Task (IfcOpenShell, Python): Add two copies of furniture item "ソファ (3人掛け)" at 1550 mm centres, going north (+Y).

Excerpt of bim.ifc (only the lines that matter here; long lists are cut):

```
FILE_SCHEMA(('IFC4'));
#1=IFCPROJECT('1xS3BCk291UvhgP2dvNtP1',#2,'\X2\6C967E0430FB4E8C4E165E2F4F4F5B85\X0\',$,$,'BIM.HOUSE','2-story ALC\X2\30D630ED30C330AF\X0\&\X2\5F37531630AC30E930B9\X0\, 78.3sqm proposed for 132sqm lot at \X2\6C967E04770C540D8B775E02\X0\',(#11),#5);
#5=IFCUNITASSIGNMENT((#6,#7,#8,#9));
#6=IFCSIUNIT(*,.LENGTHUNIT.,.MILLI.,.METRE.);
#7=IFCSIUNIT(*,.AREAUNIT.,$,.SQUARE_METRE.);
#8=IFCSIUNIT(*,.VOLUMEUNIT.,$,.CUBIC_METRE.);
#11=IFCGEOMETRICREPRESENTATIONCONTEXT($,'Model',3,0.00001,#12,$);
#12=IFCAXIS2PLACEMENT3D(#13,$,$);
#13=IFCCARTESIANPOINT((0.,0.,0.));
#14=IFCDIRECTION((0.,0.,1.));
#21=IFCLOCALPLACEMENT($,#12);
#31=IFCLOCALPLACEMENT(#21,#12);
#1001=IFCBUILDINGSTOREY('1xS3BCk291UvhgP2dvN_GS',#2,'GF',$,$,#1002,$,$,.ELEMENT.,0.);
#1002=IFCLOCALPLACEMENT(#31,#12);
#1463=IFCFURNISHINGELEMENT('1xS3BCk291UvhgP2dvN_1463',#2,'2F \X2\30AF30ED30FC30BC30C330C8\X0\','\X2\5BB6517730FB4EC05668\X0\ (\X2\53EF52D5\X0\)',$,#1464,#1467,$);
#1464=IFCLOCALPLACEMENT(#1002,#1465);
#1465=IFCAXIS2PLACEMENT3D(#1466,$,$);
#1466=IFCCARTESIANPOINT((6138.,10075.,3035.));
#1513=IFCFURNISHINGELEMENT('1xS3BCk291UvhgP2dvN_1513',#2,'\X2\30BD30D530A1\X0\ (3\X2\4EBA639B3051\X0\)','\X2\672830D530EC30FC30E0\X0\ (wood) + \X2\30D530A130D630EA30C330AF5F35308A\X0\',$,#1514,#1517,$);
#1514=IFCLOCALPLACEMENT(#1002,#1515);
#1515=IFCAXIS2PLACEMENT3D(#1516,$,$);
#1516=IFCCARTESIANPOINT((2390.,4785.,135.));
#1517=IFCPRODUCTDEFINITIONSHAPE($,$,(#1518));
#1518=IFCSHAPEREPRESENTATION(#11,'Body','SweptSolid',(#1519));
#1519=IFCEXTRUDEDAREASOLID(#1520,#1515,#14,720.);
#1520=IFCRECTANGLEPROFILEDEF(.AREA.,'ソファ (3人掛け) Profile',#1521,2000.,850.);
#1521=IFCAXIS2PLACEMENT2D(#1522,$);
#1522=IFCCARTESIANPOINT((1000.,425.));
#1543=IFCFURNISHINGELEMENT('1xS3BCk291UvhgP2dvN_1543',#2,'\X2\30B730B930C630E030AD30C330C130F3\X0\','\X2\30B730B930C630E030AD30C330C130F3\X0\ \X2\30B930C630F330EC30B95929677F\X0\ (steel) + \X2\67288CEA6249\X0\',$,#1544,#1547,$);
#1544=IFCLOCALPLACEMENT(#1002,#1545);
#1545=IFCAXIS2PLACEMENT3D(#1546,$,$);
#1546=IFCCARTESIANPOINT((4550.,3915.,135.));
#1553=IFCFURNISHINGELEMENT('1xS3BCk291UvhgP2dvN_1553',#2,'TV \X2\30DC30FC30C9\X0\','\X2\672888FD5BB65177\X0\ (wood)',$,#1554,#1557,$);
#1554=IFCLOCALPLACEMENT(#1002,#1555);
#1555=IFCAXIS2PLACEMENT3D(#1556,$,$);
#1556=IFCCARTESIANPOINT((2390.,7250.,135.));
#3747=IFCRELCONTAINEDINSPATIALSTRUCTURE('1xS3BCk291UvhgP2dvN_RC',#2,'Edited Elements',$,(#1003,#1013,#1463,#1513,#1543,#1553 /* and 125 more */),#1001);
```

```python
import numpy as np
import ifcopenshell
import ifcopenshell.api.geometry
import ifcopenshell.api.root
import ifcopenshell.util.element
import ifcopenshell.util.placement

model = ifcopenshell.open("bim.ifc")


def reuse_history(source, copy):
    """copy_class also copies each property set's owner history, people and application; keep the originals."""
    for rel in copy.IsDefinedBy:
        if rel.is_a("IfcRelDefinesByProperties") and (history := rel.RelatingPropertyDefinition.OwnerHistory):
            rel.RelatingPropertyDefinition.OwnerHistory = source.OwnerHistory
            ifcopenshell.util.element.remove_deep2(model, history)


source = model.by_guid("1xS3BCk291UvhgP2dvN_1513")
base = ifcopenshell.util.placement.get_local_placement(source.ObjectPlacement)
step = np.array([0.0, 1.0, 0.0]) * 1550.0

for i in range(1, 3):
    copy = ifcopenshell.api.root.copy_class(model, product=source)
    copy.Representation = ifcopenshell.util.element.copy_deep(
        model, source.Representation, exclude=["IfcGeometricRepresentationContext", "IfcRepresentationMap"]
    )
    reuse_history(source, copy)
    matrix = base.copy()
    matrix[:3, 3] += i * step
    print("added at", matrix[:3, 3].round(3) + 0.0)
    ifcopenshell.api.geometry.edit_object_placement(model, product=copy, matrix=matrix, is_si=False)

model.write("bim_rev.ifc")
```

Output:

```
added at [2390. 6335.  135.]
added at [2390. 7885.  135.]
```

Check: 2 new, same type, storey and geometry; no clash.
